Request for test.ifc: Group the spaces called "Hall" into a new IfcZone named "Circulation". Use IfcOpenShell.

First a look at what the model holds.

```python
import ifcopenshell

model = ifcopenshell.open("test.ifc")
print(model.schema)
seen = {}
for space in model.by_type("IfcSpace"):
    seen[space.LongName] = seen.get(space.LongName, 0) + 1
for name, count in sorted(seen.items(), key=str):
    print(count, "x", name)
print("zones:", [z.Name for z in model.by_type("IfcZone")][:20])
```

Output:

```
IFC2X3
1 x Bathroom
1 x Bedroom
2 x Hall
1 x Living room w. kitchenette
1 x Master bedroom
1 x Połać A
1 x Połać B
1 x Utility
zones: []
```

```python
import ifcopenshell
import ifcopenshell.api.group
import ifcopenshell.api.root

model = ifcopenshell.open("test.ifc")

names = {"Hall"}
spaces = [s for s in model.by_type("IfcSpace") if s.LongName in names]

zone = ifcopenshell.api.root.create_entity(model, ifc_class="IfcZone", name="Circulation")
ifcopenshell.api.group.assign_group(model, products=spaces, group=zone)
print(len(spaces), "spaces in", zone.Name)

model.write("test_updated.ifc")
```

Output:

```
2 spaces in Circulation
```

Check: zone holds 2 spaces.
